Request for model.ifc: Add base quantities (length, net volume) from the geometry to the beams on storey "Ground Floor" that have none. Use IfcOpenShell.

First a look at what the model holds.

```python
import ifcopenshell
import ifcopenshell.util.element
import ifcopenshell.util.unit

model = ifcopenshell.open("model.ifc")
print(model.schema)
for unit_type in ("LENGTHUNIT", "AREAUNIT", "VOLUMEUNIT"):
    print(unit_type, ifcopenshell.util.unit.calculate_unit_scale(model, unit_type))
storey = next(s for s in model.by_type("IfcBuildingStorey") if s.Name == "Ground Floor")
beams = [e for e in ifcopenshell.util.element.get_decomposition(storey) if e.is_a("IfcBeam")]
for e in sorted(beams, key=lambda e: e.id()):
    print(e.id(), e.is_a(), e.Name, list(ifcopenshell.util.element.get_psets(e, qtos_only=True)), sep=" | ")
```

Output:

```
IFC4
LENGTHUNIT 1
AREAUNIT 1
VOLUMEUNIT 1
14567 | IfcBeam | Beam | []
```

```python
import ifcopenshell
import ifcopenshell.api.pset
import ifcopenshell.geom
import ifcopenshell.util.element
import ifcopenshell.util.shape
import ifcopenshell.util.unit

model = ifcopenshell.open("model.ifc")
unit_scale = ifcopenshell.util.unit.calculate_unit_scale(model)
volume_scale = ifcopenshell.util.unit.calculate_unit_scale(model, "VOLUMEUNIT")
settings = ifcopenshell.geom.settings()

storey = next(s for s in model.by_type("IfcBuildingStorey") if s.Name == "Ground Floor")
beams = [e for e in ifcopenshell.util.element.get_decomposition(storey) if e.is_a("IfcBeam")]

for e in sorted(beams, key=lambda e: e.id()):
    if ifcopenshell.util.element.get_psets(e, qtos_only=True, should_inherit=False):
        continue
    # Geometry comes back in metres, in the element's own axes.
    shape = ifcopenshell.geom.create_shape(settings, e)
    values = {
        "Length": ifcopenshell.util.shape.get_max_xyz(shape.geometry) / unit_scale,
        "NetVolume": ifcopenshell.util.shape.get_volume(shape.geometry) / volume_scale,
    }
    qto = ifcopenshell.api.pset.add_qto(model, product=e, name="Qto_BeamBaseQuantities")
    ifcopenshell.api.pset.edit_qto(model, qto=qto, properties=values)
    print(e.id(), {k: round(v, 3) for k, v in values.items()})

model.write("model_edited.ifc")
```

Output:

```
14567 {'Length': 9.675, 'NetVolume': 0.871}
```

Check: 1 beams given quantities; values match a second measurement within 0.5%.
